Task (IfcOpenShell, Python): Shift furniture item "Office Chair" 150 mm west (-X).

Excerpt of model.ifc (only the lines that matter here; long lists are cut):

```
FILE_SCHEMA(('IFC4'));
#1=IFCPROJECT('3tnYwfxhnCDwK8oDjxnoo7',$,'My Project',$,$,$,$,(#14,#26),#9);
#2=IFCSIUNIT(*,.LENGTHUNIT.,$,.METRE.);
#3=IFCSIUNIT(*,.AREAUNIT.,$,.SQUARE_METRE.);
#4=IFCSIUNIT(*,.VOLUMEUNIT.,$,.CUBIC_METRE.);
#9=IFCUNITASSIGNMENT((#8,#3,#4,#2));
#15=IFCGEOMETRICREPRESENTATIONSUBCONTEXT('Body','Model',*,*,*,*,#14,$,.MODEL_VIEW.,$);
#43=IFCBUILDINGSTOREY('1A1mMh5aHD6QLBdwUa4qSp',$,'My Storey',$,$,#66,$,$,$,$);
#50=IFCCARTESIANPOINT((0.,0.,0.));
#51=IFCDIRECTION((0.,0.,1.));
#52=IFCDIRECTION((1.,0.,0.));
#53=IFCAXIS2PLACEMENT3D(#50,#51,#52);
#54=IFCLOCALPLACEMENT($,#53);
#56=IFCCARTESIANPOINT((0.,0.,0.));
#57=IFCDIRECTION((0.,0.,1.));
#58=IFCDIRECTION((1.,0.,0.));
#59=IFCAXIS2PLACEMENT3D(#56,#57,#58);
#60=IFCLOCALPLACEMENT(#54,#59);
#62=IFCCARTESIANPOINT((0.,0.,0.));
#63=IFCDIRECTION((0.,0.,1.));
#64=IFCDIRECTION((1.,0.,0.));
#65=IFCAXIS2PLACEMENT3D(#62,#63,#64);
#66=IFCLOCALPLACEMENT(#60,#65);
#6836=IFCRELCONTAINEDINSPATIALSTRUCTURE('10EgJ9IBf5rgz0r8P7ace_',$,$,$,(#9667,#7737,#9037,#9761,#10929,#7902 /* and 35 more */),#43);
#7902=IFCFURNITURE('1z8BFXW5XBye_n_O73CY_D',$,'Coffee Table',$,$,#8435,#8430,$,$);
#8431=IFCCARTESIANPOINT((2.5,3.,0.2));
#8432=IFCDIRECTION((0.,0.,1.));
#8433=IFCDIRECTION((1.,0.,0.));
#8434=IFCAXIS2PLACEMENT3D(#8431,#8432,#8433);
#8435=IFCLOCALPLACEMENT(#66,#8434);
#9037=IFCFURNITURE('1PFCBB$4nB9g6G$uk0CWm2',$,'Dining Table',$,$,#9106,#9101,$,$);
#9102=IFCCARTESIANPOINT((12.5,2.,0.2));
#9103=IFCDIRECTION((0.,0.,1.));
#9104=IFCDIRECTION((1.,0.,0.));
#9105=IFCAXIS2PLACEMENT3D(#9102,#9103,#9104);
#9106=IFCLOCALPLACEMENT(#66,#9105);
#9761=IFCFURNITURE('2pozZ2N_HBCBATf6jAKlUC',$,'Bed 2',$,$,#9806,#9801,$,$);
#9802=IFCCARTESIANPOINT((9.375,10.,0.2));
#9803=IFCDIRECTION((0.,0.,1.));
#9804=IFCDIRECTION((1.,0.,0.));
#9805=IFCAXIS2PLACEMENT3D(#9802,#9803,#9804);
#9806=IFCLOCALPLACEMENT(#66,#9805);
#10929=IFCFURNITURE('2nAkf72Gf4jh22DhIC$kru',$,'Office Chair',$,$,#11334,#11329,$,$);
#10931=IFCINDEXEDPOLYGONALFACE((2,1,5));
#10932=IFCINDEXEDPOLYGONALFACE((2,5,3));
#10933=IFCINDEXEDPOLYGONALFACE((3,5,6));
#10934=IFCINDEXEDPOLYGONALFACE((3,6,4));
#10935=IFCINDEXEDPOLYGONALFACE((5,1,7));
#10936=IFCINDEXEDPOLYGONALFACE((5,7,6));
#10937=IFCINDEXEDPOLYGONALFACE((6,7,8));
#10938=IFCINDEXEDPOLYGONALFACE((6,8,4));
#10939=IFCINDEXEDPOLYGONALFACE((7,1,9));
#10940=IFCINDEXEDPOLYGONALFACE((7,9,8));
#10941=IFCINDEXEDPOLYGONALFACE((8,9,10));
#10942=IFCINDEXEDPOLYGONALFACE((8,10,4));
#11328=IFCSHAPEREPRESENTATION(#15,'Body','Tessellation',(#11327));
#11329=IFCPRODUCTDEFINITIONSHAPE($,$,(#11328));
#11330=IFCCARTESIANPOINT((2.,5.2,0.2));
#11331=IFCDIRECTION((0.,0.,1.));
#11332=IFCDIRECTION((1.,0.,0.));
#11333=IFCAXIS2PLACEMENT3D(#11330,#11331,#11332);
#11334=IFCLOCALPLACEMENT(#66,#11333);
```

```python
import ifcopenshell
import ifcopenshell.api.geometry
import ifcopenshell.util.placement
import ifcopenshell.util.unit

model = ifcopenshell.open("model.ifc")
unit_scale = ifcopenshell.util.unit.calculate_unit_scale(model)

item = model.by_guid("2nAkf72Gf4jh22DhIC$kru")
matrix = ifcopenshell.util.placement.get_local_placement(item.ObjectPlacement)
matrix[0, 3] -= 0.15 / unit_scale
ifcopenshell.api.geometry.edit_object_placement(model, product=item, matrix=matrix, is_si=False)

print(ifcopenshell.util.placement.get_local_placement(item.ObjectPlacement).round(3) + 0.0)

model.write("model_v2.ifc")
```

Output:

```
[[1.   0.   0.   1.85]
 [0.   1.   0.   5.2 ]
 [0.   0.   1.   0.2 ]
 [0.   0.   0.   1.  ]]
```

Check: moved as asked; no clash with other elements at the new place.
